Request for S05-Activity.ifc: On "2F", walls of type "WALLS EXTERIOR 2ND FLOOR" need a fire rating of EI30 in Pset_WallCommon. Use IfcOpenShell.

First a look at what the model holds.

```python
import ifcopenshell
import ifcopenshell.util.element

model = ifcopenshell.open("S05-Activity.ifc")
print(model.schema)
storey = next(s for s in model.by_type("IfcBuildingStorey") if s.Name == "2F")
walls = [e for e in ifcopenshell.util.element.get_decomposition(storey) if e.is_a("IfcWall")]
seen = {}
for e in walls:
    element_type = ifcopenshell.util.element.get_type(e)
    key = (element_type.Name if element_type != e and element_type else None, ifcopenshell.util.element.get_pset(e, "Pset_WallCommon", "FireRating"))
    seen[key] = seen.get(key, 0) + 1
for (name, value), count in sorted(seen.items(), key=str):
    print(count, "x", name, "|", value)
```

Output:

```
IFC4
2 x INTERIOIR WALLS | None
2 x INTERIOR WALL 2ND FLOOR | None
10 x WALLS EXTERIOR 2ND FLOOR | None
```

```python
import ifcopenshell
import ifcopenshell.api.pset
import ifcopenshell.util.element

model = ifcopenshell.open("S05-Activity.ifc")

storey = next(s for s in model.by_type("IfcBuildingStorey") if s.Name == "2F")
walls = [e for e in ifcopenshell.util.element.get_decomposition(storey) if e.is_a("IfcWall")]

count = 0
for e in walls:
    element_type = ifcopenshell.util.element.get_type(e)
    if element_type in (None, e) or element_type.Name != "WALLS EXTERIOR 2ND FLOOR":
        continue
    # add_pset returns the element's existing set when there is one.
    pset = ifcopenshell.api.pset.add_pset(model, product=e, name="Pset_WallCommon")
    ifcopenshell.api.pset.edit_pset(model, pset=pset, properties={"FireRating": "EI30"})
    count += 1

print(count, "walls updated")

model.write("S05-Activity_updated.ifc")
```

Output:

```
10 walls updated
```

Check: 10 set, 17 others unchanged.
